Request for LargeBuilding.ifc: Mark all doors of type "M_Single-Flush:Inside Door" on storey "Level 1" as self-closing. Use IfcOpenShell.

First a look at what the model holds.

```python
import ifcopenshell
import ifcopenshell.util.element

model = ifcopenshell.open("LargeBuilding.ifc")
print(model.schema)
storey = next(s for s in model.by_type("IfcBuildingStorey") if s.Name == "Level 1")
doors = [e for e in ifcopenshell.util.element.get_decomposition(storey) if e.is_a("IfcDoor")]
seen = {}
for e in doors:
    element_type = ifcopenshell.util.element.get_type(e)
    key = (element_type.Name if element_type != e and element_type else None, ifcopenshell.util.element.get_pset(e, "Pset_DoorCommon", "SelfClosing"))
    seen[key] = seen.get(key, 0) + 1
for (name, value), count in sorted(seen.items(), key=str):
    print(count, "x", name, "|", value)
```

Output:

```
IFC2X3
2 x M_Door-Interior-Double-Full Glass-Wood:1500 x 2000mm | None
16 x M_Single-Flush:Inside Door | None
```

```python
import ifcopenshell
import ifcopenshell.api.pset
import ifcopenshell.util.element

model = ifcopenshell.open("LargeBuilding.ifc")

storey = next(s for s in model.by_type("IfcBuildingStorey") if s.Name == "Level 1")
doors = [e for e in ifcopenshell.util.element.get_decomposition(storey) if e.is_a("IfcDoor")]

count = 0
for e in doors:
    element_type = ifcopenshell.util.element.get_type(e)
    if element_type in (None, e) or element_type.Name != "M_Single-Flush:Inside Door":
        continue
    # add_pset returns the element's existing set when there is one.
    pset = ifcopenshell.api.pset.add_pset(model, product=e, name="Pset_DoorCommon")
    ifcopenshell.api.pset.edit_pset(model, pset=pset, properties={"SelfClosing": True})
    count += 1

print(count, "doors updated")

model.write("LargeBuilding-out.ifc")
```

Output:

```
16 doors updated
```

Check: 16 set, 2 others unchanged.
